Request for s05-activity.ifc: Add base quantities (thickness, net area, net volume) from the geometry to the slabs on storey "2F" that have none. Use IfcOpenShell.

First a look at what the model holds.

```python
import ifcopenshell
import ifcopenshell.util.element
import ifcopenshell.util.unit

model = ifcopenshell.open("s05-activity.ifc")
print(model.schema)
for unit_type in ("LENGTHUNIT", "AREAUNIT", "VOLUMEUNIT"):
    print(unit_type, ifcopenshell.util.unit.calculate_unit_scale(model, unit_type))
storey = next(s for s in model.by_type("IfcBuildingStorey") if s.Name == "2F")
slabs = [e for e in ifcopenshell.util.element.get_decomposition(storey) if e.is_a("IfcSlab")]
for e in sorted(slabs, key=lambda e: e.id()):
    print(e.id(), e.is_a(), e.Name, list(ifcopenshell.util.element.get_psets(e, qtos_only=True)), sep=" | ")
```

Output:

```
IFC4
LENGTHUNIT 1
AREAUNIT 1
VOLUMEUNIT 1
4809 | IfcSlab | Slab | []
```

```python
import ifcopenshell
import ifcopenshell.api.pset
import ifcopenshell.geom
import ifcopenshell.util.element
import ifcopenshell.util.shape
import ifcopenshell.util.unit

model = ifcopenshell.open("s05-activity.ifc")
unit_scale = ifcopenshell.util.unit.calculate_unit_scale(model)
area_scale = ifcopenshell.util.unit.calculate_unit_scale(model, "AREAUNIT")
volume_scale = ifcopenshell.util.unit.calculate_unit_scale(model, "VOLUMEUNIT")
settings = ifcopenshell.geom.settings()

storey = next(s for s in model.by_type("IfcBuildingStorey") if s.Name == "2F")
slabs = [e for e in ifcopenshell.util.element.get_decomposition(storey) if e.is_a("IfcSlab")]

for e in sorted(slabs, key=lambda e: e.id()):
    if ifcopenshell.util.element.get_psets(e, qtos_only=True, should_inherit=False):
        continue
    # Geometry comes back in metres, in the element's own axes.
    shape = ifcopenshell.geom.create_shape(settings, e)
    values = {
        "Width": ifcopenshell.util.shape.get_z(shape.geometry) / unit_scale,
        "NetArea": ifcopenshell.util.shape.get_footprint_area(shape.geometry) / area_scale,
        "NetVolume": ifcopenshell.util.shape.get_volume(shape.geometry) / volume_scale,
    }
    qto = ifcopenshell.api.pset.add_qto(model, product=e, name="Qto_SlabBaseQuantities")
    ifcopenshell.api.pset.edit_qto(model, qto=qto, properties=values)
    print(e.id(), {k: round(v, 3) for k, v in values.items()})

model.write("s05-activity_rev.ifc")
```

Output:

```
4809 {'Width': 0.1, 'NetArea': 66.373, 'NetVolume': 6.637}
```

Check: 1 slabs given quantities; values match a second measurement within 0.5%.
